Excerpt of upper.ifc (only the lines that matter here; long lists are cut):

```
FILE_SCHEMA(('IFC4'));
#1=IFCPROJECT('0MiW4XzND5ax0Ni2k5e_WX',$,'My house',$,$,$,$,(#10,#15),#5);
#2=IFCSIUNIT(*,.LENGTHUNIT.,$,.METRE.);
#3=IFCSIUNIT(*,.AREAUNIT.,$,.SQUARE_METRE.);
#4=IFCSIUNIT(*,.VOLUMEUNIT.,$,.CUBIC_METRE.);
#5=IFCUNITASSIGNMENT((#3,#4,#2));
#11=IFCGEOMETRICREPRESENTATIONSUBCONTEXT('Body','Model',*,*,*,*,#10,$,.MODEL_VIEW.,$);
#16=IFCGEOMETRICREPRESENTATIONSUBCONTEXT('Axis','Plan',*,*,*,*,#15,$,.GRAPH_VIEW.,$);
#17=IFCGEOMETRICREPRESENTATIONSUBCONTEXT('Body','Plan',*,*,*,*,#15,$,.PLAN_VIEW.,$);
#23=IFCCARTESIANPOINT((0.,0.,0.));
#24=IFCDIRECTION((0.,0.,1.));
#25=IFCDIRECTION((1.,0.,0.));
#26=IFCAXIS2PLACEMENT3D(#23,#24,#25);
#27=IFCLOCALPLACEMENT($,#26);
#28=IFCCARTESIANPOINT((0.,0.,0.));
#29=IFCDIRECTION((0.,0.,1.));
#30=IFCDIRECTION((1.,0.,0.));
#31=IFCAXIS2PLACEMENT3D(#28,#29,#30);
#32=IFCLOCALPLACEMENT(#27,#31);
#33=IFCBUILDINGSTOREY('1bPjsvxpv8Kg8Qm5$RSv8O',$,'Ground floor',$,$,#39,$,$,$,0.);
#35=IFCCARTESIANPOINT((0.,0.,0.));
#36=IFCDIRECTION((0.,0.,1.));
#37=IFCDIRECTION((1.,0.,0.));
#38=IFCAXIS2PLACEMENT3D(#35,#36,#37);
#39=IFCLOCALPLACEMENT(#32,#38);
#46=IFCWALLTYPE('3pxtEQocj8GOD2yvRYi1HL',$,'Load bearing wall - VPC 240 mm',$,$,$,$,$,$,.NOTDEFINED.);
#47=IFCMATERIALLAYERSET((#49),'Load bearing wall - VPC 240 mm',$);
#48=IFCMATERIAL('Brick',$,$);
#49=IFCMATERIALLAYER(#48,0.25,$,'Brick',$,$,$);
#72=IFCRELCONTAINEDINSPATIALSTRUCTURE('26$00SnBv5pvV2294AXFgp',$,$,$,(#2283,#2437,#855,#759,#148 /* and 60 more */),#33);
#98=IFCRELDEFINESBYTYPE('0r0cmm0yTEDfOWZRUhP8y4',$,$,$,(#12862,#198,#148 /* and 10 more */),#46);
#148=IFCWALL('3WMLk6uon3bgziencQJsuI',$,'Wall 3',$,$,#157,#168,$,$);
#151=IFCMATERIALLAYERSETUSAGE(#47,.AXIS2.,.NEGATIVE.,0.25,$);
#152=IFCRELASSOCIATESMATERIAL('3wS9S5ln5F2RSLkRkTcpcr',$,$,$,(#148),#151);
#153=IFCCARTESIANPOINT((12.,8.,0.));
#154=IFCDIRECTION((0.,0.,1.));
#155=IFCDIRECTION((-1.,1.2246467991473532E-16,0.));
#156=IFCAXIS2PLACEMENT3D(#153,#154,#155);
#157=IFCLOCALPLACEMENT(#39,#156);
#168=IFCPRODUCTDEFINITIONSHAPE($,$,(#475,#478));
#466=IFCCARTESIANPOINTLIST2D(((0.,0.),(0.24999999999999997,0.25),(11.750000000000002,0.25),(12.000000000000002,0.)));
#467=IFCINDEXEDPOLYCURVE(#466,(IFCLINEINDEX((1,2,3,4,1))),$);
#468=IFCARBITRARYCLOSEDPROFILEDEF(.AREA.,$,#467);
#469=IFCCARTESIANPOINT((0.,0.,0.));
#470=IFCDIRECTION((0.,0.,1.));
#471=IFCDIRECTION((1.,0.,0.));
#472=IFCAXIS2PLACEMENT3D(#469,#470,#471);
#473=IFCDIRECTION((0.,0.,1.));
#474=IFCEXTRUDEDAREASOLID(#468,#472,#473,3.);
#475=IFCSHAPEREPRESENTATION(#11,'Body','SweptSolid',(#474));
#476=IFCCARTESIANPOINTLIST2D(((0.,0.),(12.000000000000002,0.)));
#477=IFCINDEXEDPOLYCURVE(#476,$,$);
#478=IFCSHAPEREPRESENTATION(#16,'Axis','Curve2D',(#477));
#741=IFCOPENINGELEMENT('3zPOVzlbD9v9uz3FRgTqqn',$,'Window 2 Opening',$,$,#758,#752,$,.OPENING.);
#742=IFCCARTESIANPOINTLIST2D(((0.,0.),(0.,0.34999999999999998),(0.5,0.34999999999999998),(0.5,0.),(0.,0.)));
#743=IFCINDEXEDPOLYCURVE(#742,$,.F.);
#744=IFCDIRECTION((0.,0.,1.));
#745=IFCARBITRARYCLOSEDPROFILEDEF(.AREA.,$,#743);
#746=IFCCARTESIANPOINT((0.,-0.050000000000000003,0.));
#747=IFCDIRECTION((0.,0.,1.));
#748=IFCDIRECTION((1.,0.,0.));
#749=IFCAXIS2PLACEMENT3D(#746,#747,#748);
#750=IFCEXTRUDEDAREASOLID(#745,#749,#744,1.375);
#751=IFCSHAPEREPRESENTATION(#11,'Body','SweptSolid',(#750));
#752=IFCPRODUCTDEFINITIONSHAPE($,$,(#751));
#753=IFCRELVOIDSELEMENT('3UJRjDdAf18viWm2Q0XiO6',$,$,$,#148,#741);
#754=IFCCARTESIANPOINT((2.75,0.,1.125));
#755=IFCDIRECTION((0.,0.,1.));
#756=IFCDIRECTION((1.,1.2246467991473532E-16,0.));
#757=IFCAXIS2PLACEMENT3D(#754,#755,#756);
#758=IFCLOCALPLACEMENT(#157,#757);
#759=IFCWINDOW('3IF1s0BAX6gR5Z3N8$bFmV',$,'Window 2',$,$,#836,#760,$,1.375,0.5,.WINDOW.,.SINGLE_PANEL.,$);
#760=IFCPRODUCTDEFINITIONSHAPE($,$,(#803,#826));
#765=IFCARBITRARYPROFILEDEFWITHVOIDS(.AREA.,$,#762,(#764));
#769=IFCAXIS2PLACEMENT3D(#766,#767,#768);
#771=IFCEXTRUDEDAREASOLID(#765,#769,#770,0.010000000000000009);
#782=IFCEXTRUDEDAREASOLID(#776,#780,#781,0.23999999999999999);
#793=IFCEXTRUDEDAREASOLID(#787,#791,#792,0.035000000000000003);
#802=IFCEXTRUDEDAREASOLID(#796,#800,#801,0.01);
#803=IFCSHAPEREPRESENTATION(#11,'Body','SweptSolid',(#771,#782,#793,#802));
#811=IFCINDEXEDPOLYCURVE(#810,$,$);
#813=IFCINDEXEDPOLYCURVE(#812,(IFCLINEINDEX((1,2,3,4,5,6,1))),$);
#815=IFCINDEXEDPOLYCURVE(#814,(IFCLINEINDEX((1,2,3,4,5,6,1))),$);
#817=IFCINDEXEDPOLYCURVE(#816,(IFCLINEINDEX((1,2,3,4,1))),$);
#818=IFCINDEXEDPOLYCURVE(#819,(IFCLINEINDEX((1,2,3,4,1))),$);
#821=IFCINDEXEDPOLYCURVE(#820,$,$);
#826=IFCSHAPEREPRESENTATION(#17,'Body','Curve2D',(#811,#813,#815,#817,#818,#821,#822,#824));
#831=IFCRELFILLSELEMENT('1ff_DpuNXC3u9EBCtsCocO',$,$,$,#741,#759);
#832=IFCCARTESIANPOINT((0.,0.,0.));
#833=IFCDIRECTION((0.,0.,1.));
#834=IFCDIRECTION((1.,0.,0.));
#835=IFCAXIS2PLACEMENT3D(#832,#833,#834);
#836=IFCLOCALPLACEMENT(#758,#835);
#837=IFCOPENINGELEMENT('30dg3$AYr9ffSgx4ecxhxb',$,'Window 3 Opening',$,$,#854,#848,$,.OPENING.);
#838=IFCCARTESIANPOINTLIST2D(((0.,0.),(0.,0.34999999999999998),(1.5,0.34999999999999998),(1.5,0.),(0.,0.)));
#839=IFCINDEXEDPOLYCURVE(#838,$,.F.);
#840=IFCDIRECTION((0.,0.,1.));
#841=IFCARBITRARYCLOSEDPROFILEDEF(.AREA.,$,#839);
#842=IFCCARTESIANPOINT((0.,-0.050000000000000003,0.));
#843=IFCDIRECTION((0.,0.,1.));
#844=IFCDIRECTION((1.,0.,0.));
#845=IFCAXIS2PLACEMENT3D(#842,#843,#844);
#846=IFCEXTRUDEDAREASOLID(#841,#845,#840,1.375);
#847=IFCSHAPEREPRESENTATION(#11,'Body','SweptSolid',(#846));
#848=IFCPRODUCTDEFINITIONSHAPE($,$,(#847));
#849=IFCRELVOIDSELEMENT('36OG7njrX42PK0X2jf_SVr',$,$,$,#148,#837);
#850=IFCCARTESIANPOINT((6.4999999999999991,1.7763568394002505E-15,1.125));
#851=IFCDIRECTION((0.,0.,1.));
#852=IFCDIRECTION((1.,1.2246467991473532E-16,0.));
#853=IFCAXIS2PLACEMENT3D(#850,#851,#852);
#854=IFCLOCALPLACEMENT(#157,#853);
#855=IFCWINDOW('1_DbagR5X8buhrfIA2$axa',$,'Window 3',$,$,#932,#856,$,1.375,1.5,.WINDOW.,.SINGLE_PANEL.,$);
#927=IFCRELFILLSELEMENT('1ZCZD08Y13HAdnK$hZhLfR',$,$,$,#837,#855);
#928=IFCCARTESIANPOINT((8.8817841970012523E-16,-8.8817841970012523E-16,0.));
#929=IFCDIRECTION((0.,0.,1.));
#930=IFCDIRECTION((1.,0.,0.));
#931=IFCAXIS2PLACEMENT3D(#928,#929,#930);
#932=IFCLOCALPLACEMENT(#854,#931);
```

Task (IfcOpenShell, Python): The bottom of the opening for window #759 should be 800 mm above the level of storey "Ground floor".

```python
import numpy as np
import ifcopenshell
import ifcopenshell.api.geometry
import ifcopenshell.geom
import ifcopenshell.util.element
import ifcopenshell.util.placement
import ifcopenshell.util.shape
import ifcopenshell.util.unit

model = ifcopenshell.open("upper.ifc")
unit_scale = ifcopenshell.util.unit.calculate_unit_scale(model)

window = model.by_guid("3IF1s0BAX6gR5Z3N8$bFmV")
opening = window.FillsVoids[0].RelatingOpeningElement
storey = ifcopenshell.util.element.get_container(window, ifc_class="IfcBuildingStorey")
level = ifcopenshell.util.placement.get_local_placement(storey.ObjectPlacement)[2, 3]

# The opening's origin need not be at the sill, so measure its lowest point.
shape = ifcopenshell.geom.create_shape(ifcopenshell.geom.settings(), opening)
bottom = ifcopenshell.util.shape.get_shape_bottom_elevation(shape, shape.geometry) / unit_scale
dz = level + 0.8 - bottom

shift = np.array([0.0, 0.0, dz])
# The window is placed relative to its opening, so it follows when the opening moves.
matrix = ifcopenshell.util.placement.get_local_placement(opening.ObjectPlacement)
matrix[:3, 3] += shift
ifcopenshell.api.geometry.edit_object_placement(
    model, product=opening, matrix=matrix, is_si=False, should_transform_children=True
)

print(f"moved by {dz * unit_scale:+.3f} m")

model.write("upper_updated.ifc")
```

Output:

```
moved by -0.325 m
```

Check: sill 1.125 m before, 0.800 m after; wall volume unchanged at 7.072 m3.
